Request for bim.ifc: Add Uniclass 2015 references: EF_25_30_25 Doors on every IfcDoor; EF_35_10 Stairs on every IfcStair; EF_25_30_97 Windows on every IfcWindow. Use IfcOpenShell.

First a look at what the model holds.

```python
import ifcopenshell

model = ifcopenshell.open("bim.ifc")
print(model.schema)
print("classifications:", [c.Name for c in model.by_type("IfcClassification")])
for ifc_class in ("IfcDoor", "IfcRoof", "IfcStair", "IfcWall", "IfcWindow"):
    print(ifc_class, len(model.by_type(ifc_class)))
```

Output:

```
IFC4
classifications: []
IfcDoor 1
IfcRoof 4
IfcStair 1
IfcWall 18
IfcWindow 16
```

```python
import ifcopenshell
import ifcopenshell.api.classification

model = ifcopenshell.open("bim.ifc")

system = ifcopenshell.api.classification.add_classification(model, classification="Uniclass 2015")

codes = {
    "IfcDoor": ("EF_25_30_25", "Doors"),
    "IfcStair": ("EF_35_10", "Stairs"),
    "IfcWindow": ("EF_25_30_97", "Windows"),
}
for ifc_class, (code, name) in codes.items():
    products = model.by_type(ifc_class)
    ifcopenshell.api.classification.add_reference(
        model, products=products, classification=system, identification=code, name=name
    )
    print(code, len(products))

model.write("bim_updated.ifc")
```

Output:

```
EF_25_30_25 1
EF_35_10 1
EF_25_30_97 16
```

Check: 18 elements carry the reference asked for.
